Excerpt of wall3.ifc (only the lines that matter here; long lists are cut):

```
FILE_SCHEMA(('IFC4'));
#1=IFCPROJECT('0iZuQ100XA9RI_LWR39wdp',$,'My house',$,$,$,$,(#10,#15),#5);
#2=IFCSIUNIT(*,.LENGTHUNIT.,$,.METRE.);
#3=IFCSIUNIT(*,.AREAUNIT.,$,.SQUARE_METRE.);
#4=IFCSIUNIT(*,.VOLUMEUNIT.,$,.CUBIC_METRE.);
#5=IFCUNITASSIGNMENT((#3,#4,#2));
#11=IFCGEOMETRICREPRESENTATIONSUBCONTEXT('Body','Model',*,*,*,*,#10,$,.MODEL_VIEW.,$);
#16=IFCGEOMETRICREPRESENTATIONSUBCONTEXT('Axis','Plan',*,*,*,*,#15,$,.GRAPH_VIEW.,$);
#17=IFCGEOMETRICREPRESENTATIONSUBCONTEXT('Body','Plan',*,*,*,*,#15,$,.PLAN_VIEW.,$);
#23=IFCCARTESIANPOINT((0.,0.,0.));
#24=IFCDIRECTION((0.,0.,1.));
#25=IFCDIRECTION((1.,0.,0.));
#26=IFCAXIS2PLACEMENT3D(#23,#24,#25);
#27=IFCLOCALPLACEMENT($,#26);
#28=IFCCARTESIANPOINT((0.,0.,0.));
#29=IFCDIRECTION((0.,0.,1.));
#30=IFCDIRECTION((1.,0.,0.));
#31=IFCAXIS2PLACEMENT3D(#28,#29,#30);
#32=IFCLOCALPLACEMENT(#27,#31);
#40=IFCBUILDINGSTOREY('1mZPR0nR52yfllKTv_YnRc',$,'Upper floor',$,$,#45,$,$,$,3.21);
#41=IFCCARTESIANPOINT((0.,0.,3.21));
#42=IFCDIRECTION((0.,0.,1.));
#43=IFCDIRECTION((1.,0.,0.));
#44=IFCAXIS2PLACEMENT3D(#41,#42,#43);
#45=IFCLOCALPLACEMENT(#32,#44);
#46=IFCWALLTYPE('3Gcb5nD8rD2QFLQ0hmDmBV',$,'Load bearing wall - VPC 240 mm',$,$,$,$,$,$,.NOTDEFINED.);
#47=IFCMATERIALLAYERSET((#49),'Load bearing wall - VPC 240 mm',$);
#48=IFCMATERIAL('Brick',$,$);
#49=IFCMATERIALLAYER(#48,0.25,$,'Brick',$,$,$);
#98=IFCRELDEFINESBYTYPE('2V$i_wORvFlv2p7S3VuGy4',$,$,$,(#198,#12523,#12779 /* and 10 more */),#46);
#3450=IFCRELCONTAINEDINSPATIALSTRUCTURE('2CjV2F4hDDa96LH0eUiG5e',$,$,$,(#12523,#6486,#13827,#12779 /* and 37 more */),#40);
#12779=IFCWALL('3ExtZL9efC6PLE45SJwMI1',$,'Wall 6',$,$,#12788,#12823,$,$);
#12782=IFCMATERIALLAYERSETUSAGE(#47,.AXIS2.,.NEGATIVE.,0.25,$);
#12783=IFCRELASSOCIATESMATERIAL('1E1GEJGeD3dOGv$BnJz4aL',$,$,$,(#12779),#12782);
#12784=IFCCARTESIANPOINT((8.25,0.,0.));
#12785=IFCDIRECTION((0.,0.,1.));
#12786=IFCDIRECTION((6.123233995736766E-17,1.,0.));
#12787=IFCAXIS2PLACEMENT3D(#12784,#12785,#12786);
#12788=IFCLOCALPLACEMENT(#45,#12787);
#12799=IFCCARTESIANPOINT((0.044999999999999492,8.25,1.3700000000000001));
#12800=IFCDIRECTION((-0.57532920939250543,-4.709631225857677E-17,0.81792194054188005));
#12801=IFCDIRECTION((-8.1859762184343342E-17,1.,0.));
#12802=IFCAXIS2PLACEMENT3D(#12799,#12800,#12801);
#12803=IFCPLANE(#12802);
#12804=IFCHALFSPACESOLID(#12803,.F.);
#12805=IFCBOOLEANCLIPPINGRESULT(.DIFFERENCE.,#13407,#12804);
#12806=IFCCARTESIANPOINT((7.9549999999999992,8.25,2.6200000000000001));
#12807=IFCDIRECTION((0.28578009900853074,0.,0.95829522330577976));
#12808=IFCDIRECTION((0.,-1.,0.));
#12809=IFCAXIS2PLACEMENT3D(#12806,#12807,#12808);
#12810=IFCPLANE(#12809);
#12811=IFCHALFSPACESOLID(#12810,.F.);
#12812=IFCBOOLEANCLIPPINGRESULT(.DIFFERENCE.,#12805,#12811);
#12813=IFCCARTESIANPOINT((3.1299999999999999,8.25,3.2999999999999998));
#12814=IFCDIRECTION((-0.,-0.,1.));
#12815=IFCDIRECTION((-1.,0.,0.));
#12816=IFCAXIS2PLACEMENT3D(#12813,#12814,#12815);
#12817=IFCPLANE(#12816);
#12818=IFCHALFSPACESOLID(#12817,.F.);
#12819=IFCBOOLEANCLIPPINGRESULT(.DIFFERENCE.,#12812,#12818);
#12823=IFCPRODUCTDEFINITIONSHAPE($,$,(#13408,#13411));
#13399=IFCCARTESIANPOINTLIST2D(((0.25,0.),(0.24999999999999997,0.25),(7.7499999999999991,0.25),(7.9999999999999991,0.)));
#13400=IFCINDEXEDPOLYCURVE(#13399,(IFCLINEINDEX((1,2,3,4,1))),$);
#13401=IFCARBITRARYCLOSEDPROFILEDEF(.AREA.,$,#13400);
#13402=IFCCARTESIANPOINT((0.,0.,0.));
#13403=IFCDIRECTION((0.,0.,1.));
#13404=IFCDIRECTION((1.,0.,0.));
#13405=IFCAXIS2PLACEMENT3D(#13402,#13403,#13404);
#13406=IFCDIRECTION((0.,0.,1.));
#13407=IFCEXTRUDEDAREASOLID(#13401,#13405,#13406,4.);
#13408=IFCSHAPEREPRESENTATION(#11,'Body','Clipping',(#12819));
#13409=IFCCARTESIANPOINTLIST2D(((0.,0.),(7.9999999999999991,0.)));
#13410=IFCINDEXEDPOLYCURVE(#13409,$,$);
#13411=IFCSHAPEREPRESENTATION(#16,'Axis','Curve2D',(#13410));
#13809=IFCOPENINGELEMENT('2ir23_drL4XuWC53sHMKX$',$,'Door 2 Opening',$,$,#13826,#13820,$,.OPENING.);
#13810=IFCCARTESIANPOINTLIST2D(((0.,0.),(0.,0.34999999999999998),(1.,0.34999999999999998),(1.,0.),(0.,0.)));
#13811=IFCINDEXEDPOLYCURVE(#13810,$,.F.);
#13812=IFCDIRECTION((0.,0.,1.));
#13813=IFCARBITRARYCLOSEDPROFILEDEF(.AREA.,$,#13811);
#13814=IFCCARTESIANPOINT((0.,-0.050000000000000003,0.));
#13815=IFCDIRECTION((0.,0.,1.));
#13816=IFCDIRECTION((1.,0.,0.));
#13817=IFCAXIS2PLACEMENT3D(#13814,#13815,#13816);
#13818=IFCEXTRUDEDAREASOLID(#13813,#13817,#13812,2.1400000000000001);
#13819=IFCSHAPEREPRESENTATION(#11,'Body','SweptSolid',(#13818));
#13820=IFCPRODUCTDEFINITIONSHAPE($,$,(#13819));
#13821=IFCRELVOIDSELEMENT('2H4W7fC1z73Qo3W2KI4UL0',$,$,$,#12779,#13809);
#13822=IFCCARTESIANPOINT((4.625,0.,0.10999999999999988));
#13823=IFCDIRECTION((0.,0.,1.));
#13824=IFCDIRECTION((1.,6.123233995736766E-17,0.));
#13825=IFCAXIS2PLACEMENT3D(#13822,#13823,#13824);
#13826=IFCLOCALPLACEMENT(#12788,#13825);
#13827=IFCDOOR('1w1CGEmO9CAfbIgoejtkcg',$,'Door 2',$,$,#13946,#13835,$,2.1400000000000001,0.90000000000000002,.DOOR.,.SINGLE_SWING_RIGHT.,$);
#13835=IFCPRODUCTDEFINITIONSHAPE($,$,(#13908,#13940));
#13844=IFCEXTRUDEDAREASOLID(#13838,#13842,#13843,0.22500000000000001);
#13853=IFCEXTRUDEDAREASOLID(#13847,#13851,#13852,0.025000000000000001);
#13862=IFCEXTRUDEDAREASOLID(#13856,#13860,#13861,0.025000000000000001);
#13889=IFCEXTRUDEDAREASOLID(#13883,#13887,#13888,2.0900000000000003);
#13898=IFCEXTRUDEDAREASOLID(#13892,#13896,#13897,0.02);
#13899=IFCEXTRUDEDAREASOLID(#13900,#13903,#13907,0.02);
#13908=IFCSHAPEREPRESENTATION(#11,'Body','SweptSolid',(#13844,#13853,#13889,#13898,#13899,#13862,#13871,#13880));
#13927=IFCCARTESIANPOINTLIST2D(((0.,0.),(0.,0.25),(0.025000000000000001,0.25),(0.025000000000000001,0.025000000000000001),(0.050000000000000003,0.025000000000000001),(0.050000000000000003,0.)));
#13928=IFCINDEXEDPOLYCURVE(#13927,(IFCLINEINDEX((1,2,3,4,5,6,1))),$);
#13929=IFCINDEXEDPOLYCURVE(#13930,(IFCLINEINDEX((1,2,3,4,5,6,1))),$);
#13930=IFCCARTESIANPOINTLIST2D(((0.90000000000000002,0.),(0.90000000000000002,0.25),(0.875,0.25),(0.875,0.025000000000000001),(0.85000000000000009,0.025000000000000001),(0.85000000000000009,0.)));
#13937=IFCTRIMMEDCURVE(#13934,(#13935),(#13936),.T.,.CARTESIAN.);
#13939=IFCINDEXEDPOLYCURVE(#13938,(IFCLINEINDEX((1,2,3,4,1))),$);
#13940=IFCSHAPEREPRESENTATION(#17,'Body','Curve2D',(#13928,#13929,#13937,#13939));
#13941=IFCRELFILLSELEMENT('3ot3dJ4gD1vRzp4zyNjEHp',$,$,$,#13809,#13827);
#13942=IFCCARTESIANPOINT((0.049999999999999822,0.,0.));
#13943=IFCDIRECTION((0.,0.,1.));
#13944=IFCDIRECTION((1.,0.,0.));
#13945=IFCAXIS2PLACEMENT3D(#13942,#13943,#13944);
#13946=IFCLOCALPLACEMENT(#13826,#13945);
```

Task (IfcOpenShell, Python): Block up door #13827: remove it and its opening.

```python
import ifcopenshell
import ifcopenshell.api.feature
import ifcopenshell.api.root
import ifcopenshell.geom
import ifcopenshell.util.shape

model = ifcopenshell.open("wall3.ifc")
settings = ifcopenshell.geom.settings()


def volume(element):
    """Net volume in cubic metres, openings subtracted."""
    shape = ifcopenshell.geom.create_shape(settings, element)
    return ifcopenshell.util.shape.get_volume(shape.geometry)


door = model.by_guid("1w1CGEmO9CAfbIgoejtkcg")
opening = door.FillsVoids[0].RelatingOpeningElement
wall = opening.VoidsElements[0].RelatingBuildingElement
before = volume(wall)

ifcopenshell.api.root.remove_product(model, product=door)
ifcopenshell.api.feature.remove_feature(model, feature=opening)

after = volume(wall)

print(f"wall volume {before:.3f} -> {after:.3f} m3")

model.write("wall3-out.ifc")
```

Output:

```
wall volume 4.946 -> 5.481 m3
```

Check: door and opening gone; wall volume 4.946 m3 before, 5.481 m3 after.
